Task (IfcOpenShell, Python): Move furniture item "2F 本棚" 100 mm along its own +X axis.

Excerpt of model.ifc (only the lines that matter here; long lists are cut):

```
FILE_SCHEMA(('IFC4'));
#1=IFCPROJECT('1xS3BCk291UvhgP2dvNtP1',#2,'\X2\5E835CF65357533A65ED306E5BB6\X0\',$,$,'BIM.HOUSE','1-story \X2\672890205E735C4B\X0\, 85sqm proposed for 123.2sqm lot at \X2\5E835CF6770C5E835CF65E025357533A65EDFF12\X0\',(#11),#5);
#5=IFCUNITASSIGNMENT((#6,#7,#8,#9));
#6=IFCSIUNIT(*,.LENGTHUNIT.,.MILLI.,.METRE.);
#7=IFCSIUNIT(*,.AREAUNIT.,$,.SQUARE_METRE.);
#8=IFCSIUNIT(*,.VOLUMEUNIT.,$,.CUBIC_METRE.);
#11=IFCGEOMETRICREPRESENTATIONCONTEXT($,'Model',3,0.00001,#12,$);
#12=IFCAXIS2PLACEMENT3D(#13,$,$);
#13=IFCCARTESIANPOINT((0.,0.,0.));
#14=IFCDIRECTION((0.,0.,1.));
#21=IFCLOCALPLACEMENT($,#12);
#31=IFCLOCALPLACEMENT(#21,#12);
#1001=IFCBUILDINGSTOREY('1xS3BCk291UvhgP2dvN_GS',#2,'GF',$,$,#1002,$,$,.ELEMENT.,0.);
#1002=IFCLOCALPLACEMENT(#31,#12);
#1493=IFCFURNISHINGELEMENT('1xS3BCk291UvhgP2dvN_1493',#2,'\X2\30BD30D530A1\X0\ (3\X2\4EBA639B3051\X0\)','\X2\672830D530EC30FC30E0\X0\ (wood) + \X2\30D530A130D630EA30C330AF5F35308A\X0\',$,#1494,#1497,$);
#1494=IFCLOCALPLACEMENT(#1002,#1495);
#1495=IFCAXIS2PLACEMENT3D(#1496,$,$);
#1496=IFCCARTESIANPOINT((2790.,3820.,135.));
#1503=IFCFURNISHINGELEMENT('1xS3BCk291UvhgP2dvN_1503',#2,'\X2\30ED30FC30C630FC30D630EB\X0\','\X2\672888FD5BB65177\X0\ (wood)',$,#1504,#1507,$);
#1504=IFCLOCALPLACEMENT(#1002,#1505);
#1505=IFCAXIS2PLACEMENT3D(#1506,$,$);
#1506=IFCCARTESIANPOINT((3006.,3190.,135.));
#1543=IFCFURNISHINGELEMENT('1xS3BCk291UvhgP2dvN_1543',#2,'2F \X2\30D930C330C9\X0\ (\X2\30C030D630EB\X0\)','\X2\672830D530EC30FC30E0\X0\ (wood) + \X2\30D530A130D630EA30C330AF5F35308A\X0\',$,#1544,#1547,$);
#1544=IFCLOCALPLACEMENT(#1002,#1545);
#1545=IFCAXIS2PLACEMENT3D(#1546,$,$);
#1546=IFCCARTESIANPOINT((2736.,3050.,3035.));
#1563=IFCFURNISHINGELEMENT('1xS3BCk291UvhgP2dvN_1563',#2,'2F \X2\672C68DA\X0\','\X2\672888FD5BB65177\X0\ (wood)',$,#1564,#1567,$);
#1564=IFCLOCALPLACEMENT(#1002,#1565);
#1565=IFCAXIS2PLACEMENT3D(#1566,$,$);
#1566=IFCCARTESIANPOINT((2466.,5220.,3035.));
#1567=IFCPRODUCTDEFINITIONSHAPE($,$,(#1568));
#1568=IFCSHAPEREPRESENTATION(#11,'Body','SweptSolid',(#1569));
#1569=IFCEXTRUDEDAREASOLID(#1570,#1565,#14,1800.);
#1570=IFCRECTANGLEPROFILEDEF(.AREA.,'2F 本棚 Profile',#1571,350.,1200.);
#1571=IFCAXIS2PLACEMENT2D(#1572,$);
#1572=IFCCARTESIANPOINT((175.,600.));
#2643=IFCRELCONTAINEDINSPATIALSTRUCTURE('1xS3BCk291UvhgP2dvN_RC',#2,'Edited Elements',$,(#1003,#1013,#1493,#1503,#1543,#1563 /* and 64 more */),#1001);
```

```python
import ifcopenshell
import ifcopenshell.api.geometry
import ifcopenshell.util.placement
import ifcopenshell.util.unit

model = ifcopenshell.open("model.ifc")
unit_scale = ifcopenshell.util.unit.calculate_unit_scale(model)

item = model.by_id(1563)
matrix = ifcopenshell.util.placement.get_local_placement(item.ObjectPlacement)
matrix[:3, 3] += matrix[:3, 0] * 0.1 / unit_scale
ifcopenshell.api.geometry.edit_object_placement(model, product=item, matrix=matrix, is_si=False)

print(ifcopenshell.util.placement.get_local_placement(item.ObjectPlacement).round(3) + 0.0)

model.write("model_rev.ifc")
```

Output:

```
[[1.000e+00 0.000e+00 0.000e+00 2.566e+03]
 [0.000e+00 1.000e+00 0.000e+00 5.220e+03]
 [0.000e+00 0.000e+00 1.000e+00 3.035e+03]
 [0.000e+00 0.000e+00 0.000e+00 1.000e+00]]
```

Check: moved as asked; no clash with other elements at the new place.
